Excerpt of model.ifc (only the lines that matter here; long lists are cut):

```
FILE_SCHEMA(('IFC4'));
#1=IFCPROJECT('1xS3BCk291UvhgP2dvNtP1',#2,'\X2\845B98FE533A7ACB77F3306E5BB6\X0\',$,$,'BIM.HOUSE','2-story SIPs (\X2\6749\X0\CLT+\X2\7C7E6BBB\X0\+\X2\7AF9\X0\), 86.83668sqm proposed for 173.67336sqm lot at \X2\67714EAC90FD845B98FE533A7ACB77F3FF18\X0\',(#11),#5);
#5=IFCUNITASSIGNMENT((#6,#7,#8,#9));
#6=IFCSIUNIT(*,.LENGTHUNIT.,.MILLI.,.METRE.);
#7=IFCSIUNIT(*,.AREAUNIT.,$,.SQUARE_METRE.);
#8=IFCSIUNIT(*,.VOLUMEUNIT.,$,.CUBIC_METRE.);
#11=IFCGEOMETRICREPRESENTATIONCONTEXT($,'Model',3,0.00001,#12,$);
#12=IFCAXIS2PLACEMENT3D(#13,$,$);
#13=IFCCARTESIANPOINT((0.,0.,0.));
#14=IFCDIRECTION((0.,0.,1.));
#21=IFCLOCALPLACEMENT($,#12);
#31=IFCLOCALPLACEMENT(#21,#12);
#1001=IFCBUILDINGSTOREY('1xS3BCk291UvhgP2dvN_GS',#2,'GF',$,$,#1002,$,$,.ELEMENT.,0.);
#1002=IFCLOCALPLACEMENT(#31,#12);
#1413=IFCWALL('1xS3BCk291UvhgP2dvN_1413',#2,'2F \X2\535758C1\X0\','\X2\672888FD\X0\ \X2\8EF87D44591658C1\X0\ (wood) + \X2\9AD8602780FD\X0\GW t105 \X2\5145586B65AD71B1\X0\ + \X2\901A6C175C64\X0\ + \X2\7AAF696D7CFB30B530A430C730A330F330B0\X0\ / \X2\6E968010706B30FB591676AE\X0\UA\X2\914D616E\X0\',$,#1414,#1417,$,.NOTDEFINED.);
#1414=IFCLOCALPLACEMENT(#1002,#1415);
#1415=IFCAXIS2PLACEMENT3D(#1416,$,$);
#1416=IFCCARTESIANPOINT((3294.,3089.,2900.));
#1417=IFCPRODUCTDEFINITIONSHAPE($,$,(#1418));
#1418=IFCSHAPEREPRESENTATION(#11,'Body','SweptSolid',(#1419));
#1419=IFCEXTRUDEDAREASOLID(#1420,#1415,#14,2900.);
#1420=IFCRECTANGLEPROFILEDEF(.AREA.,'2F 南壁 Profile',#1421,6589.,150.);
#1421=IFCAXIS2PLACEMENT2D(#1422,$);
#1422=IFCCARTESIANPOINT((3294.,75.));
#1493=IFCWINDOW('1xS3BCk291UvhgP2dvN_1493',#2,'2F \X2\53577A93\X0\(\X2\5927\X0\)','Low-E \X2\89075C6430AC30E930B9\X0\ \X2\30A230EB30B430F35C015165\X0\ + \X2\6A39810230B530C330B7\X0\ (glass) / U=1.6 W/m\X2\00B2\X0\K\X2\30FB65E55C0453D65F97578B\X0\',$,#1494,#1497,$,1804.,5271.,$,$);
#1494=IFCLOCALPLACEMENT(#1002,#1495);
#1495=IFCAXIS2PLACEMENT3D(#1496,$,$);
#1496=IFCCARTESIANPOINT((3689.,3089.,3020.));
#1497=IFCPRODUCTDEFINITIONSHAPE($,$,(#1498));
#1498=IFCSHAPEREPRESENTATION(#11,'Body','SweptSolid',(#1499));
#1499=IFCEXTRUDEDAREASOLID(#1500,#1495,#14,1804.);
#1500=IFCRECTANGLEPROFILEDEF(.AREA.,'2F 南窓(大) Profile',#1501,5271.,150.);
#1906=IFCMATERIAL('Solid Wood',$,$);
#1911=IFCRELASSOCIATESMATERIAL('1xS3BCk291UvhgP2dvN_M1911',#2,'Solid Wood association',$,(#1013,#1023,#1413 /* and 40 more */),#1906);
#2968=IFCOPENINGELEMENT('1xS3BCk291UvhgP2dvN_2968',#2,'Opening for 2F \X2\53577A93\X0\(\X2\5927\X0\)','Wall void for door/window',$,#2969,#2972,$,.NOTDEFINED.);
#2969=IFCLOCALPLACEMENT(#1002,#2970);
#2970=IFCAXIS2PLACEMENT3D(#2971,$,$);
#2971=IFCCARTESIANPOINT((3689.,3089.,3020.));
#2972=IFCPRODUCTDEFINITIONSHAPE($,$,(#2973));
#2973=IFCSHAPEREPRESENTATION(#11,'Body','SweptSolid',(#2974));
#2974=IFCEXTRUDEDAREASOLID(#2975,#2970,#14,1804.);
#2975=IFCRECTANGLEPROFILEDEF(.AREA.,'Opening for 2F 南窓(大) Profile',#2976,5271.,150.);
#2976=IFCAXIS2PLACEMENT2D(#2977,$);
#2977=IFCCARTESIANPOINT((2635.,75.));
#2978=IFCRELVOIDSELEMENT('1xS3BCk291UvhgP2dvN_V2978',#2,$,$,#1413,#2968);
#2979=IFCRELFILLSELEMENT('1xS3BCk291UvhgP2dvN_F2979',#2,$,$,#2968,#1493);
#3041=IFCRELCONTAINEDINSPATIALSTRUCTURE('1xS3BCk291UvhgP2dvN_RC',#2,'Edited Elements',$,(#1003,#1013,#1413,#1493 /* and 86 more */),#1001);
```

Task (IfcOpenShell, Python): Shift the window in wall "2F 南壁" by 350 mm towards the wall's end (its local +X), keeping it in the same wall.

```python
import ifcopenshell
import ifcopenshell.api.geometry
import ifcopenshell.util.placement

model = ifcopenshell.open("model.ifc")

window = model.by_guid("1xS3BCk291UvhgP2dvN_1493")
opening = window.FillsVoids[0].RelatingOpeningElement
wall = opening.VoidsElements[0].RelatingBuildingElement

wall_matrix = ifcopenshell.util.placement.get_local_placement(wall.ObjectPlacement)
shift = wall_matrix[:3, 0] * 350.0
before = ifcopenshell.util.placement.get_local_placement(window.ObjectPlacement)[:3, 3].copy()

# The window is not placed relative to its opening, so move both.
for product in (opening, window):
    matrix = ifcopenshell.util.placement.get_local_placement(product.ObjectPlacement)
    matrix[:3, 3] += shift
    ifcopenshell.api.geometry.edit_object_placement(model, product=product, matrix=matrix, is_si=False)

after = ifcopenshell.util.placement.get_local_placement(window.ObjectPlacement)[:3, 3]
print("window moved by", (after - before).round(3) + 0.0)

model.write("model_rev.ifc")
```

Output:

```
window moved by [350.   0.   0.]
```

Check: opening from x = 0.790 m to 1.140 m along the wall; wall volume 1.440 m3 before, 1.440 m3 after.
